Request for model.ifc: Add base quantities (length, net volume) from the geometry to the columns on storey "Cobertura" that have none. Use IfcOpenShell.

First a look at what the model holds.

```python
import ifcopenshell
import ifcopenshell.util.element
import ifcopenshell.util.unit

model = ifcopenshell.open("model.ifc")
print(model.schema)
for unit_type in ("LENGTHUNIT", "AREAUNIT", "VOLUMEUNIT"):
    print(unit_type, ifcopenshell.util.unit.calculate_unit_scale(model, unit_type))
storey = next(s for s in model.by_type("IfcBuildingStorey") if s.Name == "Cobertura")
columns = [e for e in ifcopenshell.util.element.get_decomposition(storey) if e.is_a("IfcColumn")]
for e in sorted(columns, key=lambda e: e.id()):
    print(e.id(), e.is_a(), e.Name, list(ifcopenshell.util.element.get_psets(e, qtos_only=True)), sep=" | ")
```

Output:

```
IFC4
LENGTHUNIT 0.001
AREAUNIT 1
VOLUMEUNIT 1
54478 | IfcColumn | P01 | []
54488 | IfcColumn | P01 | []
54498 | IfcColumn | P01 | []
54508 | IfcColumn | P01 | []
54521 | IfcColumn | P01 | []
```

```python
import ifcopenshell
import ifcopenshell.api.pset
import ifcopenshell.geom
import ifcopenshell.util.element
import ifcopenshell.util.shape
import ifcopenshell.util.unit

model = ifcopenshell.open("model.ifc")
unit_scale = ifcopenshell.util.unit.calculate_unit_scale(model)
volume_scale = ifcopenshell.util.unit.calculate_unit_scale(model, "VOLUMEUNIT")
settings = ifcopenshell.geom.settings()

storey = next(s for s in model.by_type("IfcBuildingStorey") if s.Name == "Cobertura")
columns = [e for e in ifcopenshell.util.element.get_decomposition(storey) if e.is_a("IfcColumn")]

for e in sorted(columns, key=lambda e: e.id()):
    if ifcopenshell.util.element.get_psets(e, qtos_only=True, should_inherit=False):
        continue
    # Geometry comes back in metres, in the element's own axes.
    shape = ifcopenshell.geom.create_shape(settings, e)
    values = {
        "Length": ifcopenshell.util.shape.get_z(shape.geometry) / unit_scale,
        "NetVolume": ifcopenshell.util.shape.get_volume(shape.geometry) / volume_scale,
    }
    qto = ifcopenshell.api.pset.add_qto(model, product=e, name="Qto_ColumnBaseQuantities")
    ifcopenshell.api.pset.edit_qto(model, qto=qto, properties=values)
    print(e.id(), {k: round(v, 3) for k, v in values.items()})

model.write("model_updated.ifc")
```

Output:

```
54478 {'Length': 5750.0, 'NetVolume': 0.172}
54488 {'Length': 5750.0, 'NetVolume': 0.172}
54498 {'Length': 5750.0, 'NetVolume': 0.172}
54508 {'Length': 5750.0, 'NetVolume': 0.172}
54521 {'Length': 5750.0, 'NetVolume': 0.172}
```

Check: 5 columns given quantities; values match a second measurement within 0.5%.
